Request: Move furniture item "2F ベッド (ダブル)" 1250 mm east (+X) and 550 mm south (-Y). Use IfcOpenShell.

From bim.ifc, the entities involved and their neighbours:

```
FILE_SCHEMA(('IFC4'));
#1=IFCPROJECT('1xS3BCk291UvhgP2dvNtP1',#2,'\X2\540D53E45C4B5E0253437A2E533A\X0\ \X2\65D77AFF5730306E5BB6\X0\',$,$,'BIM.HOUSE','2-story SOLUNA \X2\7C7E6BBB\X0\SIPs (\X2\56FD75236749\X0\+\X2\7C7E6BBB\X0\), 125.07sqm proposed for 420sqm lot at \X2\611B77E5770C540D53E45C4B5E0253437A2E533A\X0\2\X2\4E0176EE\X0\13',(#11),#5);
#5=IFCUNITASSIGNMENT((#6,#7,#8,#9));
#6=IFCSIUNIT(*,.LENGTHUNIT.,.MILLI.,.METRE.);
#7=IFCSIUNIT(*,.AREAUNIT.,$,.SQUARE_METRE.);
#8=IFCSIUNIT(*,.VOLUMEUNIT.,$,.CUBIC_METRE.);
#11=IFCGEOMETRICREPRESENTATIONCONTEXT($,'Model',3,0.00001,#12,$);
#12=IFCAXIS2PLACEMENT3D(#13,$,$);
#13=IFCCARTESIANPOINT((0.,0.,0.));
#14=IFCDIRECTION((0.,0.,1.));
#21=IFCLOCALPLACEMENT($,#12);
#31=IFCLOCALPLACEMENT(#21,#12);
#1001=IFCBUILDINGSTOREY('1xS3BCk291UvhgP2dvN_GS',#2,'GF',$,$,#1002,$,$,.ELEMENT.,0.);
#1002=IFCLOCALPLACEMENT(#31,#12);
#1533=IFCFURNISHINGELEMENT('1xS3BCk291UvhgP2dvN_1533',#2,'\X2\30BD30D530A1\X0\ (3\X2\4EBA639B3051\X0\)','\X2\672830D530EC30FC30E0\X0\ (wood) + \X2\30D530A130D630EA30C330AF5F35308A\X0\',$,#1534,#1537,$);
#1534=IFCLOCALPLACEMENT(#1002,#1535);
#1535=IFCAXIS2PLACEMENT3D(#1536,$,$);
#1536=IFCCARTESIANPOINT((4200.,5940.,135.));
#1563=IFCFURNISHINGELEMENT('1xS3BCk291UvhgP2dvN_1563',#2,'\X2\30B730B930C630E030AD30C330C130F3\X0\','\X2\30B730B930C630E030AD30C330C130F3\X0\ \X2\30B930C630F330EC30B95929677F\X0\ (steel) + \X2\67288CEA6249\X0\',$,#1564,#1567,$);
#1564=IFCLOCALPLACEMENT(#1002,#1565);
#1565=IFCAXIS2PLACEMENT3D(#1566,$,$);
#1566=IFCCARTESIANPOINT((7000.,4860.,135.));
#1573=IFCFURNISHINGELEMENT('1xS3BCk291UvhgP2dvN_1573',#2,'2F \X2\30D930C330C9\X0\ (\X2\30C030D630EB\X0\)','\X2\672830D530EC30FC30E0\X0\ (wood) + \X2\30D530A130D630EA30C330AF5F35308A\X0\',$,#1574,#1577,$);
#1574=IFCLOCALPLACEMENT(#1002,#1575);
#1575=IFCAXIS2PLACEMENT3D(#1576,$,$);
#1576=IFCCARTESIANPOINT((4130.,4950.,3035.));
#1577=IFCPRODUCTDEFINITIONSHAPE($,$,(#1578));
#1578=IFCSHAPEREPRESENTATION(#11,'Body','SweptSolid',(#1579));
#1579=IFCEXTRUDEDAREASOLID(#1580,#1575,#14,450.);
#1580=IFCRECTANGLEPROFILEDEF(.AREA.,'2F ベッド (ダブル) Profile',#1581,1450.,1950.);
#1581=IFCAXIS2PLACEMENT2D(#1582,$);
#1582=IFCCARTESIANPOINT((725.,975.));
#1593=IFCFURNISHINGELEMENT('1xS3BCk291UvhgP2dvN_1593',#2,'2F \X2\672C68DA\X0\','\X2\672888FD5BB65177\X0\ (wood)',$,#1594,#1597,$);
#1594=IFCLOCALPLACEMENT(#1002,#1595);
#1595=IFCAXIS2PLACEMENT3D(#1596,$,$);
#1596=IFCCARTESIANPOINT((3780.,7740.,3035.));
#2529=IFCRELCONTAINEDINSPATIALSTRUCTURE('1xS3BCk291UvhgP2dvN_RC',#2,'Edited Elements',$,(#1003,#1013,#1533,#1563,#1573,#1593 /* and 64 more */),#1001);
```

```python
import ifcopenshell
import ifcopenshell.api.geometry
import ifcopenshell.util.placement

model = ifcopenshell.open("bim.ifc")

item = model.by_id(1573)
matrix = ifcopenshell.util.placement.get_local_placement(item.ObjectPlacement)
matrix[0, 3] += 1250.0
matrix[1, 3] -= 550.0
ifcopenshell.api.geometry.edit_object_placement(model, product=item, matrix=matrix, is_si=False)

print(ifcopenshell.util.placement.get_local_placement(item.ObjectPlacement).round(3) + 0.0)

model.write("bim_updated.ifc")
```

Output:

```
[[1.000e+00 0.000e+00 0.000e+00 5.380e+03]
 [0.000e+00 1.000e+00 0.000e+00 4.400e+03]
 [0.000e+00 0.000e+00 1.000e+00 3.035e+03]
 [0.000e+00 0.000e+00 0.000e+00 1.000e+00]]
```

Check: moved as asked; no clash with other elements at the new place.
